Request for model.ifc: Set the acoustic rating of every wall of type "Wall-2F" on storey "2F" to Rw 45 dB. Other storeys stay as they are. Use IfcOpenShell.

First a look at what the model holds.

```python
import ifcopenshell
import ifcopenshell.util.element

model = ifcopenshell.open("model.ifc")
print(model.schema)
storey = next(s for s in model.by_type("IfcBuildingStorey") if s.Name == "2F")
walls = [e for e in ifcopenshell.util.element.get_decomposition(storey) if e.is_a("IfcWall")]
seen = {}
for e in walls:
    element_type = ifcopenshell.util.element.get_type(e)
    key = (element_type.Name if element_type != e and element_type else None, ifcopenshell.util.element.get_pset(e, "Pset_WallCommon", "AcousticRating"))
    seen[key] = seen.get(key, 0) + 1
for (name, value), count in sorted(seen.items(), key=str):
    print(count, "x", name, "|", value)
```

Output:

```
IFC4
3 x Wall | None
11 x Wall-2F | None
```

```python
import ifcopenshell
import ifcopenshell.api.pset
import ifcopenshell.util.element

model = ifcopenshell.open("model.ifc")

storey = next(s for s in model.by_type("IfcBuildingStorey") if s.Name == "2F")
walls = [e for e in ifcopenshell.util.element.get_decomposition(storey) if e.is_a("IfcWall")]

count = 0
for e in walls:
    element_type = ifcopenshell.util.element.get_type(e)
    if element_type in (None, e) or element_type.Name != "Wall-2F":
        continue
    # add_pset returns the element's existing set when there is one.
    pset = ifcopenshell.api.pset.add_pset(model, product=e, name="Pset_WallCommon")
    ifcopenshell.api.pset.edit_pset(model, pset=pset, properties={"AcousticRating": "Rw 45 dB"})
    count += 1

print(count, "walls updated")

model.write("model_v2.ifc")
```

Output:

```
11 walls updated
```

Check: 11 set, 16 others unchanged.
